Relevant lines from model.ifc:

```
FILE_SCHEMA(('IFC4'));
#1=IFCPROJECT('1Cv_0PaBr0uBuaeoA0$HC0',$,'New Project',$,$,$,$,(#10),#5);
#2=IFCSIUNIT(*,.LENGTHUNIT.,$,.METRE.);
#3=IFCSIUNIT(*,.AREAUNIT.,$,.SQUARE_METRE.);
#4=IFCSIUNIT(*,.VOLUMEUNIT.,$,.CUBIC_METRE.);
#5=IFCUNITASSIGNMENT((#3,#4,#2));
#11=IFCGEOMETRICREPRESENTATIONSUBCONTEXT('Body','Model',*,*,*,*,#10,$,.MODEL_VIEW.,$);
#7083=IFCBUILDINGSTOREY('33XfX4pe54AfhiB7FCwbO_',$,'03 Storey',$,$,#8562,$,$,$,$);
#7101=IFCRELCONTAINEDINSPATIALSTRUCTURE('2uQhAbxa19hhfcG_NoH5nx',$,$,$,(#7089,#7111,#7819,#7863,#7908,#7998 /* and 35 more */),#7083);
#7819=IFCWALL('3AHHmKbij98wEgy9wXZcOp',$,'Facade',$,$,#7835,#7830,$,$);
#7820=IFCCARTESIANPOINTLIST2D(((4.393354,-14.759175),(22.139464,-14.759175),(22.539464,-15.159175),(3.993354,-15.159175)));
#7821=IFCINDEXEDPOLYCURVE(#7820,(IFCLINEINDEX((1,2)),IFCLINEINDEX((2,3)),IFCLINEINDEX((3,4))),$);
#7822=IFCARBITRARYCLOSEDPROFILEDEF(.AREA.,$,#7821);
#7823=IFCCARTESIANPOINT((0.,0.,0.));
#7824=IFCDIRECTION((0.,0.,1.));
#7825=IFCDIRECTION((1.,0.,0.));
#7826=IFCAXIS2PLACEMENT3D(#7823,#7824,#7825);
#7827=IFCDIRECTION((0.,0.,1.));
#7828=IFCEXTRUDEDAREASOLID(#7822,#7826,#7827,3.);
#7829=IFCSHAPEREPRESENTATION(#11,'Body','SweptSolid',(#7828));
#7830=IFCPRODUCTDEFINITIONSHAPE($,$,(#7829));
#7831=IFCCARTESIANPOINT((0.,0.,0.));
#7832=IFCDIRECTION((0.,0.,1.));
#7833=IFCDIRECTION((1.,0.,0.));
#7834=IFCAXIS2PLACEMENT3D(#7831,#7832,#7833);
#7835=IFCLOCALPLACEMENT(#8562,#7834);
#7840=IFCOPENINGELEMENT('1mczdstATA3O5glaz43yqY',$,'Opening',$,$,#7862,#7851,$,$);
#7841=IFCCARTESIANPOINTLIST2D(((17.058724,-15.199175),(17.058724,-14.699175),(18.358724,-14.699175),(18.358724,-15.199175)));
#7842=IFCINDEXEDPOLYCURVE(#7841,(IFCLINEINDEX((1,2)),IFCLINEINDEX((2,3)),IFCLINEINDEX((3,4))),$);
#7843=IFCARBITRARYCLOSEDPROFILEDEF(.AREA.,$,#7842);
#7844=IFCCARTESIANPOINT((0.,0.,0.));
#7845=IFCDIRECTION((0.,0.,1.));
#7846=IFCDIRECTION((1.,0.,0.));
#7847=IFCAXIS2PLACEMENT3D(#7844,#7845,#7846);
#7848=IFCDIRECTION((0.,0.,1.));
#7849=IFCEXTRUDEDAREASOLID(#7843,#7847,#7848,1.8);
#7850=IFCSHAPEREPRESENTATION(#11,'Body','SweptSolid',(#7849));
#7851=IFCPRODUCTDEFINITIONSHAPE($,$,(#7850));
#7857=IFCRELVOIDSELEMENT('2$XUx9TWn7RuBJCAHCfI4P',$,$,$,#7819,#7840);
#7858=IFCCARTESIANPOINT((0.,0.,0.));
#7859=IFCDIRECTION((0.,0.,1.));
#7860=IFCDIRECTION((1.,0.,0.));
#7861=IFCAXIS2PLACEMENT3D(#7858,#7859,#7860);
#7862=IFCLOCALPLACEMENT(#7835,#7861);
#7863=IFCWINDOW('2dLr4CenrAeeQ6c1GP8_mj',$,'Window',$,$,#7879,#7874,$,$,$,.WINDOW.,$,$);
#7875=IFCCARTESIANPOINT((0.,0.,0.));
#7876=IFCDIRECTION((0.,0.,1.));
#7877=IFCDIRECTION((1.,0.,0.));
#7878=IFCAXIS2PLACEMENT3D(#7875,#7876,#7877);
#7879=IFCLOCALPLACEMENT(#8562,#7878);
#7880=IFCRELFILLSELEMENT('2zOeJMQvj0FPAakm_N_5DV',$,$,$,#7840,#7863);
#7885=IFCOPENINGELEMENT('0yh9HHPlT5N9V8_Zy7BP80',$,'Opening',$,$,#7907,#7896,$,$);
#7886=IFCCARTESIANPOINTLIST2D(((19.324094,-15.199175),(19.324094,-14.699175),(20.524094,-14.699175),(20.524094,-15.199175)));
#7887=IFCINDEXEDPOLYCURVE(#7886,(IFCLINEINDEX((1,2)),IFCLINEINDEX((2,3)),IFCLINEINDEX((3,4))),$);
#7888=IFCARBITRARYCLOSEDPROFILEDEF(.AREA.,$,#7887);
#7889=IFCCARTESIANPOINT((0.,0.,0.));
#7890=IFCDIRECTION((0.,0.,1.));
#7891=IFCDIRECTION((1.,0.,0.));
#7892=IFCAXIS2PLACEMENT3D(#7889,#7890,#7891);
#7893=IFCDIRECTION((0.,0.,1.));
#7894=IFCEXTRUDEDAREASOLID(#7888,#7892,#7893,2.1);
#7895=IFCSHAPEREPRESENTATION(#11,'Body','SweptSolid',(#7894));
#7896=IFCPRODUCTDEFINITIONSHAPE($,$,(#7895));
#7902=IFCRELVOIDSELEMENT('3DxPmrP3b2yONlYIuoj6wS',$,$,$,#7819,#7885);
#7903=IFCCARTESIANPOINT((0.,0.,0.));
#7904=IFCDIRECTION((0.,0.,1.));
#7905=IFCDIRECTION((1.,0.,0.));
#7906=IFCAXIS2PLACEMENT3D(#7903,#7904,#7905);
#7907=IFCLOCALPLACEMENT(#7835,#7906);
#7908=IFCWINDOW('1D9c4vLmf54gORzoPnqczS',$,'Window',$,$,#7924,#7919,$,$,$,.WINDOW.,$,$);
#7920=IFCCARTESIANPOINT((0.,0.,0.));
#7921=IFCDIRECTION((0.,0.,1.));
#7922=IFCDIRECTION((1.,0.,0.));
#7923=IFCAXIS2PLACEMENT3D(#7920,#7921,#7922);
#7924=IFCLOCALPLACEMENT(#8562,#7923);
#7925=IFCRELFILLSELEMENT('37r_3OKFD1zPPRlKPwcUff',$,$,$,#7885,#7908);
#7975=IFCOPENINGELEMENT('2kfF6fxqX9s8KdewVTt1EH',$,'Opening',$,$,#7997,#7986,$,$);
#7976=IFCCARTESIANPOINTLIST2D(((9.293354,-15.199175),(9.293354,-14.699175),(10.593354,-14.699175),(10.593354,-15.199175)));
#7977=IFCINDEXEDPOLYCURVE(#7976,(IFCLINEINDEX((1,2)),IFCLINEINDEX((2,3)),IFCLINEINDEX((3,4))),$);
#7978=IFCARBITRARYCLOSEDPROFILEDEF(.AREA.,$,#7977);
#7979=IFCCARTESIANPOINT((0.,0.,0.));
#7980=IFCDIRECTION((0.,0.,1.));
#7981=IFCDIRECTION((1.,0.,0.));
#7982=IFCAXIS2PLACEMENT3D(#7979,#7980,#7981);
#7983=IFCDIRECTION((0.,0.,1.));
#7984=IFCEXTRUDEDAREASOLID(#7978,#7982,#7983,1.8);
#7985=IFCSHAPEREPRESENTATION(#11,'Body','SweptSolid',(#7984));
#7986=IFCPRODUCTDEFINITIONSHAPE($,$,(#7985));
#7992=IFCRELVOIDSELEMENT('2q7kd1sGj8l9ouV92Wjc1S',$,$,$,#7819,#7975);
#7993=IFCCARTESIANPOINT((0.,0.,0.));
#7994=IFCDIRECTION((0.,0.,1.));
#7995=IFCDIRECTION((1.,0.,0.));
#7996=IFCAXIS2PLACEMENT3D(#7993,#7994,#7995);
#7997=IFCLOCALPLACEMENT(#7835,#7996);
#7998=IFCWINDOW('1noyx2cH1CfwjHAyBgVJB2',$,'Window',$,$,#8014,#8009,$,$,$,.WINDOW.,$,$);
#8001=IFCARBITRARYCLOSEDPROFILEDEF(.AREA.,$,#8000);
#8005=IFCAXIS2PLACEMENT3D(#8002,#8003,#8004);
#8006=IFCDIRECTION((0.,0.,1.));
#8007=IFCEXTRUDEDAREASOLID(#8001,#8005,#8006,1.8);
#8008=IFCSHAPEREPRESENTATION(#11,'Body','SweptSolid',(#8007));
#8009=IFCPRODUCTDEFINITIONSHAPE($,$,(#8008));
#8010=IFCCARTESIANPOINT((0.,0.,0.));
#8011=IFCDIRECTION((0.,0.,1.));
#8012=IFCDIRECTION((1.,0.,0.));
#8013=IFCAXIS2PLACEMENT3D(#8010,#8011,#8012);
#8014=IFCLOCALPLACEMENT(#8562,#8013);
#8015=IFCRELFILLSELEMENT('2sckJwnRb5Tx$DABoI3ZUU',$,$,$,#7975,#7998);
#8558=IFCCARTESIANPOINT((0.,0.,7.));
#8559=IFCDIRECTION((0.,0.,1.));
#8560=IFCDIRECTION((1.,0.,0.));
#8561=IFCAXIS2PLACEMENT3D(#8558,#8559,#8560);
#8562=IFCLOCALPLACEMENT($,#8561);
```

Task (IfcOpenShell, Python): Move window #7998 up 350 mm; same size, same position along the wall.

```python
import numpy as np
import ifcopenshell
import ifcopenshell.api.geometry
import ifcopenshell.util.placement
import ifcopenshell.util.unit

model = ifcopenshell.open("model.ifc")
unit_scale = ifcopenshell.util.unit.calculate_unit_scale(model)

window = model.by_guid("1noyx2cH1CfwjHAyBgVJB2")
opening = window.FillsVoids[0].RelatingOpeningElement
dz = 0.35 / unit_scale

shift = np.array([0.0, 0.0, dz])
# The window is not placed relative to its opening, so move both.
for product in (opening, window):
    matrix = ifcopenshell.util.placement.get_local_placement(product.ObjectPlacement)
    matrix[:3, 3] += shift
    ifcopenshell.api.geometry.edit_object_placement(model, product=product, matrix=matrix, is_si=False)

print(f"moved by {dz * unit_scale:+.3f} m")

model.write("model_edited.ifc")
```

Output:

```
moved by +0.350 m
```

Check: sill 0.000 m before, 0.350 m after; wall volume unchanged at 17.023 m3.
